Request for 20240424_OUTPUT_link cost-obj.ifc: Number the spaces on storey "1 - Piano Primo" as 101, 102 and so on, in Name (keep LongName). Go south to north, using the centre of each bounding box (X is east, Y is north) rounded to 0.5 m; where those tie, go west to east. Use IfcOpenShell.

First a look at what the model holds.

```python
import ifcopenshell
import ifcopenshell.util.element
import ifcopenshell.util.placement

model = ifcopenshell.open("20240424_OUTPUT_link cost-obj.ifc")
print(model.schema)
storey = next(s for s in model.by_type("IfcBuildingStorey") if s.Name == "1 - Piano Primo")
spaces = [e for e in ifcopenshell.util.element.get_decomposition(storey) if e.is_a("IfcSpace")]
for e in sorted(spaces, key=lambda e: e.id()):
    origin = ifcopenshell.util.placement.get_local_placement(e.ObjectPlacement)[:3, 3]
    print(e.id(), e.Name, e.LongName, origin.round(2) + 0.0, sep=" | ")
```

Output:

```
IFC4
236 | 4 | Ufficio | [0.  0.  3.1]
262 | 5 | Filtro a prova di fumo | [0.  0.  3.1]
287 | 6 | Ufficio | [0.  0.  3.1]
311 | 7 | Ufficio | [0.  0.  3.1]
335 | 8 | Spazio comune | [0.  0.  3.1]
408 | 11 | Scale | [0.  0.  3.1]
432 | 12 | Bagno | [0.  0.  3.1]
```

```python
import ifcopenshell
import ifcopenshell.geom
import ifcopenshell.util.element
import ifcopenshell.util.shape

model = ifcopenshell.open("20240424_OUTPUT_link cost-obj.ifc")
settings = ifcopenshell.geom.settings()
settings.set("use-world-coords", True)


def centre(element):
    shape = ifcopenshell.geom.create_shape(settings, element)
    return ifcopenshell.util.shape.get_bbox_centroid(shape.geometry)


storey = next(s for s in model.by_type("IfcBuildingStorey") if s.Name == "1 - Piano Primo")
spaces = [e for e in ifcopenshell.util.element.get_decomposition(storey) if e.is_a("IfcSpace")]

# Insertion points can sit at a corner or the storey origin, so sort by the geometry (in metres).
centres = {e: centre(e) for e in spaces}
spaces.sort(key=lambda e: (round(centres[e][1] / 0.5), centres[e][0]))

for i, e in enumerate(spaces, start=1):
    number = f"1{i:02d}"
    e.Name = number
    print(e.id(), number)

model.write("20240424_OUTPUT_link cost-obj_v2.ifc")
```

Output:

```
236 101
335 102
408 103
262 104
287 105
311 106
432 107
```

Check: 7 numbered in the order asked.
